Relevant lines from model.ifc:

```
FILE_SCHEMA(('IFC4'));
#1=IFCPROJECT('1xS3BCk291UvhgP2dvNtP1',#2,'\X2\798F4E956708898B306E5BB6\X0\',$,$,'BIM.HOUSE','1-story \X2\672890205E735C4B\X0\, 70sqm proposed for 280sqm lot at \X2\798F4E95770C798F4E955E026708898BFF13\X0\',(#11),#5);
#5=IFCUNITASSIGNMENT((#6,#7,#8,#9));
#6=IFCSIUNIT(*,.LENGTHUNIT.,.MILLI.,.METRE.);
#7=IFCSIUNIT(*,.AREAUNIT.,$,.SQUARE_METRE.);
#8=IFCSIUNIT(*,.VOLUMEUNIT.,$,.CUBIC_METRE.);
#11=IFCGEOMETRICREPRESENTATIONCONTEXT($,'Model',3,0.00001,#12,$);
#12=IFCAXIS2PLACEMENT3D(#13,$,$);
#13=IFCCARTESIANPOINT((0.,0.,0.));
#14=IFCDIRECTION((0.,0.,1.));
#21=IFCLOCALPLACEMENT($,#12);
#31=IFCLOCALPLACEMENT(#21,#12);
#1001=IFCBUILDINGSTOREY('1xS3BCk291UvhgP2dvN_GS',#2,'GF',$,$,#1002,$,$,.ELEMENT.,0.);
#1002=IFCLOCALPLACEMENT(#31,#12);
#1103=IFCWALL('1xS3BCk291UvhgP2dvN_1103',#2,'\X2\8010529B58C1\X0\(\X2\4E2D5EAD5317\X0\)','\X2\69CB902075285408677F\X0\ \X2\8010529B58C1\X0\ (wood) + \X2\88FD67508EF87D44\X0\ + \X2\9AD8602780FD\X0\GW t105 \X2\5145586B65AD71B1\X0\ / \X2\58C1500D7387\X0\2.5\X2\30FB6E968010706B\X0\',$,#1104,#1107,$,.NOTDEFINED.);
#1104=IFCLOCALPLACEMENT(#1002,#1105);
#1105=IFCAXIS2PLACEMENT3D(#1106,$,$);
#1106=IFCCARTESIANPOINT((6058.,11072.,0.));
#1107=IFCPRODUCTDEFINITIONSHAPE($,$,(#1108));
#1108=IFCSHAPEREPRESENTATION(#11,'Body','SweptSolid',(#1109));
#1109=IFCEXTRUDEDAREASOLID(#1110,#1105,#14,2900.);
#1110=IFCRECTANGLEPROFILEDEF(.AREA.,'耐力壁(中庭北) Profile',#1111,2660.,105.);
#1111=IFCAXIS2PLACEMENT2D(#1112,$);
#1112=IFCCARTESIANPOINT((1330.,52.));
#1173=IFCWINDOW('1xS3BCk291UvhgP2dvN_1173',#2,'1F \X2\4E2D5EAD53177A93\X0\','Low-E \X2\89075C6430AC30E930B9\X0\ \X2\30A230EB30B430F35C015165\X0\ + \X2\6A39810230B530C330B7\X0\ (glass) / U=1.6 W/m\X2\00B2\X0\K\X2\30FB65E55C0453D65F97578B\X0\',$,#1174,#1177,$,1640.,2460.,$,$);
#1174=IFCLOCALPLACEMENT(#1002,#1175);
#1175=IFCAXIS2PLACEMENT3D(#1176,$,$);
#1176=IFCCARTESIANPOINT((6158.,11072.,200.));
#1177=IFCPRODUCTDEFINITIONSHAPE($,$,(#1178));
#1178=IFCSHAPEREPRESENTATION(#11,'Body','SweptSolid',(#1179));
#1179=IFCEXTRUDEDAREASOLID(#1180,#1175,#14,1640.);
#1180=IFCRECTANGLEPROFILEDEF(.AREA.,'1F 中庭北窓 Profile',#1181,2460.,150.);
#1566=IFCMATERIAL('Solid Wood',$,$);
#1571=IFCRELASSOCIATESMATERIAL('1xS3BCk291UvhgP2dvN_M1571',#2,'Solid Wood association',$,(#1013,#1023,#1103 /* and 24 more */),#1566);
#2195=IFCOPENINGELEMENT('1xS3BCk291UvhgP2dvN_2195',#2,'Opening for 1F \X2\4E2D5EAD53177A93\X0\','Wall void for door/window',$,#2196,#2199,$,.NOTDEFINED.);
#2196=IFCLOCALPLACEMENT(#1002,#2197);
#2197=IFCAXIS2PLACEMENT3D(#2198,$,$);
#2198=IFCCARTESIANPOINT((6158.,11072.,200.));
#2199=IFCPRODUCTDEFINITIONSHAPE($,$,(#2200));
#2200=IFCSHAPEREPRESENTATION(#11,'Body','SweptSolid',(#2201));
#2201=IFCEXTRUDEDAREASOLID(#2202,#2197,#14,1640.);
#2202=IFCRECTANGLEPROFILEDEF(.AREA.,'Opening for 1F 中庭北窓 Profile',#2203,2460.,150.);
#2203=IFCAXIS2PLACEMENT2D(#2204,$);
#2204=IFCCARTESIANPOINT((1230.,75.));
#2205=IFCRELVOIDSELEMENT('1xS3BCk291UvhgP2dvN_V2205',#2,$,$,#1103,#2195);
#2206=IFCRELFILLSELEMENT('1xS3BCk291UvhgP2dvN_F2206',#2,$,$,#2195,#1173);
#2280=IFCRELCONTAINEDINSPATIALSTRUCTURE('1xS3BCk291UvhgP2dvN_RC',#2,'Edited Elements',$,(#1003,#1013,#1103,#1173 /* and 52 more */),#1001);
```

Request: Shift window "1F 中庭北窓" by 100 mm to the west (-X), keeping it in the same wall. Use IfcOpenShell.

```python
import ifcopenshell
import ifcopenshell.api.geometry
import ifcopenshell.util.placement

model = ifcopenshell.open("model.ifc")

window = model.by_id(1173)
opening = window.FillsVoids[0].RelatingOpeningElement
wall = opening.VoidsElements[0].RelatingBuildingElement

wall_matrix = ifcopenshell.util.placement.get_local_placement(wall.ObjectPlacement)
shift = wall_matrix[:3, 0] * -100.0
before = ifcopenshell.util.placement.get_local_placement(window.ObjectPlacement)[:3, 3].copy()

# The window is not placed relative to its opening, so move both.
for product in (opening, window):
    matrix = ifcopenshell.util.placement.get_local_placement(product.ObjectPlacement)
    matrix[:3, 3] += shift
    ifcopenshell.api.geometry.edit_object_placement(model, product=product, matrix=matrix, is_si=False)

after = ifcopenshell.util.placement.get_local_placement(window.ObjectPlacement)[:3, 3]
print("window moved by", (after - before).round(3) + 0.0)

model.write("model_v2.ifc")
```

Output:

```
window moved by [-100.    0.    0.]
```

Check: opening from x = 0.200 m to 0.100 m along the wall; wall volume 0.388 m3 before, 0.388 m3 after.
